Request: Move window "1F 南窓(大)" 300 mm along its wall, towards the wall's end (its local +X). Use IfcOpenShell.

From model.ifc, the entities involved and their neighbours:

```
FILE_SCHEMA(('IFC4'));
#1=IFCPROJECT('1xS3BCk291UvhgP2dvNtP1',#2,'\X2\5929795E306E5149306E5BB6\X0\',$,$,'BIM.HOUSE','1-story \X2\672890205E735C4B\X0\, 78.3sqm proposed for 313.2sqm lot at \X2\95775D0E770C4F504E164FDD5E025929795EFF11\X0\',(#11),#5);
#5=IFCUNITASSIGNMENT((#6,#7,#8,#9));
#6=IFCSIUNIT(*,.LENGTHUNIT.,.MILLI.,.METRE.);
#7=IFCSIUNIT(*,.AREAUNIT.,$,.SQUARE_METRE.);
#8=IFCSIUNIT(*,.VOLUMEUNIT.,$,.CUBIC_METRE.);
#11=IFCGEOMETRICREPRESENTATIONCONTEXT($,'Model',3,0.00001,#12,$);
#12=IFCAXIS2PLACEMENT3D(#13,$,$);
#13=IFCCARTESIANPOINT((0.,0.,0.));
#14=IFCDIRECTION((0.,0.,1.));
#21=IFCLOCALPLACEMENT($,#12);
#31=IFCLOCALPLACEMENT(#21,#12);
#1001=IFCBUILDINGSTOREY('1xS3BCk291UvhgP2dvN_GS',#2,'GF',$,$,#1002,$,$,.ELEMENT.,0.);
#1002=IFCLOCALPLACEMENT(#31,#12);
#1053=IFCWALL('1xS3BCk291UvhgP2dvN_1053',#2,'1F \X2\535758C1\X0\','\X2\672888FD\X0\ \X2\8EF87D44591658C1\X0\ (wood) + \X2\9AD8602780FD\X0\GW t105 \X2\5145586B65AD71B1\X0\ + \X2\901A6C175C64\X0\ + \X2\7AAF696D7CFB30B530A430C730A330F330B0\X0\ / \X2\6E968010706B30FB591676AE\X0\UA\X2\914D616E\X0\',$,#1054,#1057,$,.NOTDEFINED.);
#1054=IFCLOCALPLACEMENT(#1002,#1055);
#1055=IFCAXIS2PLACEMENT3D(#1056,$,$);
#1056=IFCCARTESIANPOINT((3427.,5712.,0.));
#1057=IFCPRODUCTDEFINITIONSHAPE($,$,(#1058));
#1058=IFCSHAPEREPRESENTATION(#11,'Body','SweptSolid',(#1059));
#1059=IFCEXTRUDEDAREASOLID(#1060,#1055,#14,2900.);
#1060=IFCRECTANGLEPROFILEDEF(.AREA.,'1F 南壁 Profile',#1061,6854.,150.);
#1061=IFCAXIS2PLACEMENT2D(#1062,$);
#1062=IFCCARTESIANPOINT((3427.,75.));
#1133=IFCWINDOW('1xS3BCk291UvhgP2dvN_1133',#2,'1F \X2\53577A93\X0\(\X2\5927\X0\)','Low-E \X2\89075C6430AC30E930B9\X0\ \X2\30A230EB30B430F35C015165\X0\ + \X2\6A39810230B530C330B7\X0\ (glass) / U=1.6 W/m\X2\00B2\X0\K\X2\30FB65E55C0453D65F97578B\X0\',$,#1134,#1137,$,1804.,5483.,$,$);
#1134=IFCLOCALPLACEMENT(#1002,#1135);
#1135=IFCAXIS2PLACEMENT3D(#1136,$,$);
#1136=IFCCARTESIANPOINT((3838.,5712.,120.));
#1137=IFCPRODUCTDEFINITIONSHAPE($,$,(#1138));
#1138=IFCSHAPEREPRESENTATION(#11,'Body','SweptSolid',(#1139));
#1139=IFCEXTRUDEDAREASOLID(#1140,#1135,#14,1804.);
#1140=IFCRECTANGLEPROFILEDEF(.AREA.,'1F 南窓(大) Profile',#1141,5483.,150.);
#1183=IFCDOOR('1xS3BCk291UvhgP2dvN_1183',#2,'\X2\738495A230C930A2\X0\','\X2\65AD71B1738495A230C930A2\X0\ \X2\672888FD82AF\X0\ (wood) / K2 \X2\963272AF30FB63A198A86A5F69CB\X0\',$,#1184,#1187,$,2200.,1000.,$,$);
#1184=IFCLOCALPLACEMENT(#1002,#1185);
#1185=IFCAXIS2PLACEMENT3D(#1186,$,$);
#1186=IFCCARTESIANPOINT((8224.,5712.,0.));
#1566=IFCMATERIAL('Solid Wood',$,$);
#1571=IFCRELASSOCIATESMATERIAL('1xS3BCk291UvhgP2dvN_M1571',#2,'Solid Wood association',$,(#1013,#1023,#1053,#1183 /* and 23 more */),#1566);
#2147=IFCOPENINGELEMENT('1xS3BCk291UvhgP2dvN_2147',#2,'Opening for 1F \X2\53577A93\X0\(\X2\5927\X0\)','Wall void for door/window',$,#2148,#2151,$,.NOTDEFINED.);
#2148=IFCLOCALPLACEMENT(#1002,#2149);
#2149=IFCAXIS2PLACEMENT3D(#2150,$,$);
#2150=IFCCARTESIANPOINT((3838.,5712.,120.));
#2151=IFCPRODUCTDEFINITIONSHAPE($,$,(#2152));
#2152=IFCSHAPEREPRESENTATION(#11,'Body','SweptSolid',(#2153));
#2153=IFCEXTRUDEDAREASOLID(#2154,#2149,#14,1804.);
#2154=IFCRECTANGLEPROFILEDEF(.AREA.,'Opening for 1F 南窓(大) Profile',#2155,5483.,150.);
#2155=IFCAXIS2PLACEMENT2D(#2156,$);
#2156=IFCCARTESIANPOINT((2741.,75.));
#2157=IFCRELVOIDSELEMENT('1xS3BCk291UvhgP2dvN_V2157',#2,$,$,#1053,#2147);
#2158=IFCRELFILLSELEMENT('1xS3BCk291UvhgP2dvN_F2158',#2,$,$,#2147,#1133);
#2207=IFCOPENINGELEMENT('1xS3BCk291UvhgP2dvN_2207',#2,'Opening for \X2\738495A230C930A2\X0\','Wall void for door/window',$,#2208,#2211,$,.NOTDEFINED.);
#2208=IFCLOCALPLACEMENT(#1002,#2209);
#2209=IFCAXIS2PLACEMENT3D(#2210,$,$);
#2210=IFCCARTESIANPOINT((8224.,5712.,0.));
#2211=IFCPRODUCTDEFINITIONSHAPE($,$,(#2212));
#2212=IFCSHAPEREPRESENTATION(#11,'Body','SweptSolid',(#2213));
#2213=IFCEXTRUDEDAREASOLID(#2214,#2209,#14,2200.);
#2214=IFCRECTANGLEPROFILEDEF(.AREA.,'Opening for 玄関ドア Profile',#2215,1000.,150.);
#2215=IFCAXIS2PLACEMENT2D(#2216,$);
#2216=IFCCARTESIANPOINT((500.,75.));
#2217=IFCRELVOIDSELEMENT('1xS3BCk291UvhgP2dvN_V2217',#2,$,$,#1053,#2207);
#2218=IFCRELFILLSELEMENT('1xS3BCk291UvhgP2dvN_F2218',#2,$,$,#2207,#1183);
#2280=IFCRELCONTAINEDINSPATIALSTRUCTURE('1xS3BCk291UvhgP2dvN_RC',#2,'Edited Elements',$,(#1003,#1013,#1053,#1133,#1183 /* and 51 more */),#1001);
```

```python
import ifcopenshell
import ifcopenshell.api.geometry
import ifcopenshell.util.placement
import ifcopenshell.util.unit

model = ifcopenshell.open("model.ifc")
unit_scale = ifcopenshell.util.unit.calculate_unit_scale(model)

window = model.by_guid("1xS3BCk291UvhgP2dvN_1133")
opening = window.FillsVoids[0].RelatingOpeningElement
wall = opening.VoidsElements[0].RelatingBuildingElement

wall_matrix = ifcopenshell.util.placement.get_local_placement(wall.ObjectPlacement)
shift = wall_matrix[:3, 0] * 0.3 / unit_scale
before = ifcopenshell.util.placement.get_local_placement(window.ObjectPlacement)[:3, 3].copy()

# The window is not placed relative to its opening, so move both.
for product in (opening, window):
    matrix = ifcopenshell.util.placement.get_local_placement(product.ObjectPlacement)
    matrix[:3, 3] += shift
    ifcopenshell.api.geometry.edit_object_placement(model, product=product, matrix=matrix, is_si=False)

after = ifcopenshell.util.placement.get_local_placement(window.ObjectPlacement)[:3, 3]
print("window moved by", (after - before).round(3) + 0.0)

model.write("model-out.ifc")
```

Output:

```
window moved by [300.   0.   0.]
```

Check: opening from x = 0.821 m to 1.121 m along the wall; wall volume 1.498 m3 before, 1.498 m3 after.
